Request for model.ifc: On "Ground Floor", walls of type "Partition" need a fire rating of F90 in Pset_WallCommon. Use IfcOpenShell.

First a look at what the model holds.

```python
import ifcopenshell
import ifcopenshell.util.element

model = ifcopenshell.open("model.ifc")
print(model.schema)
storey = next(s for s in model.by_type("IfcBuildingStorey") if s.Name == "Ground Floor")
walls = [e for e in ifcopenshell.util.element.get_decomposition(storey) if e.is_a("IfcWall")]
seen = {}
for e in walls:
    element_type = ifcopenshell.util.element.get_type(e)
    key = (element_type.Name if element_type != e and element_type else None, ifcopenshell.util.element.get_pset(e, "Pset_WallCommon", "FireRating"))
    seen[key] = seen.get(key, 0) + 1
for (name, value), count in sorted(seen.items(), key=str):
    print(count, "x", name, "|", value)
```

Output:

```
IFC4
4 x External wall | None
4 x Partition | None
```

```python
import ifcopenshell
import ifcopenshell.api.pset
import ifcopenshell.util.element

model = ifcopenshell.open("model.ifc")

storey = next(s for s in model.by_type("IfcBuildingStorey") if s.Name == "Ground Floor")
walls = [e for e in ifcopenshell.util.element.get_decomposition(storey) if e.is_a("IfcWall")]

count = 0
for e in walls:
    element_type = ifcopenshell.util.element.get_type(e)
    if element_type in (None, e) or element_type.Name != "Partition":
        continue
    # add_pset returns the element's existing set when there is one.
    pset = ifcopenshell.api.pset.add_pset(model, product=e, name="Pset_WallCommon")
    ifcopenshell.api.pset.edit_pset(model, pset=pset, properties={"FireRating": "F90"})
    count += 1

print(count, "walls updated")

model.write("model_updated.ifc")
```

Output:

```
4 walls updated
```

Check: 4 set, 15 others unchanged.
